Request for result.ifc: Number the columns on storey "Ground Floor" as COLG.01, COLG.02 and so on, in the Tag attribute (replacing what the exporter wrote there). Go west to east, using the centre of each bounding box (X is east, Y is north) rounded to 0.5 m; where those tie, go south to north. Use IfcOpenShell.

First a look at what the model holds.

```python
import ifcopenshell
import ifcopenshell.util.element
import ifcopenshell.util.placement

model = ifcopenshell.open("result.ifc")
print(model.schema)
storey = next(s for s in model.by_type("IfcBuildingStorey") if s.Name == "Ground Floor")
columns = [e for e in ifcopenshell.util.element.get_decomposition(storey) if e.is_a("IfcColumn")]
for e in sorted(columns, key=lambda e: e.id()):
    origin = ifcopenshell.util.placement.get_local_placement(e.ObjectPlacement)[:3, 3]
    print(e.id(), e.Tag, e.Name, origin.round(2) + 0.0, sep=" | ")
```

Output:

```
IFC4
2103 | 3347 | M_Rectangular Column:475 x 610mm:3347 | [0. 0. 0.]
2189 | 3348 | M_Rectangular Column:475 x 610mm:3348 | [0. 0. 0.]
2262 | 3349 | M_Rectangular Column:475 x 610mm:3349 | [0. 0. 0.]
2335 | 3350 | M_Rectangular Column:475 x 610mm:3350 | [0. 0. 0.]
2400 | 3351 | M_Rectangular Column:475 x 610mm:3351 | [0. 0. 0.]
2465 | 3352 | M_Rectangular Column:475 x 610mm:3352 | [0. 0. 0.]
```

```python
import ifcopenshell
import ifcopenshell.geom
import ifcopenshell.util.element
import ifcopenshell.util.shape

model = ifcopenshell.open("result.ifc")
settings = ifcopenshell.geom.settings()
settings.set("use-world-coords", True)


def centre(element):
    shape = ifcopenshell.geom.create_shape(settings, element)
    return ifcopenshell.util.shape.get_bbox_centroid(shape.geometry)


storey = next(s for s in model.by_type("IfcBuildingStorey") if s.Name == "Ground Floor")
columns = [e for e in ifcopenshell.util.element.get_decomposition(storey) if e.is_a("IfcColumn")]

# Insertion points can sit at a corner or the storey origin, so sort by the geometry (in metres).
centres = {e: centre(e) for e in columns}
columns.sort(key=lambda e: (round(centres[e][0] / 0.5), centres[e][1]))

for i, e in enumerate(columns, start=1):
    number = f"COLG.{i:02d}"
    e.Tag = number
    print(e.id(), number)

model.write("result_updated.ifc")
```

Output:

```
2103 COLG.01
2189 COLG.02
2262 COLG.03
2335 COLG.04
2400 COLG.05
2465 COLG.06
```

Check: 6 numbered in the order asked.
